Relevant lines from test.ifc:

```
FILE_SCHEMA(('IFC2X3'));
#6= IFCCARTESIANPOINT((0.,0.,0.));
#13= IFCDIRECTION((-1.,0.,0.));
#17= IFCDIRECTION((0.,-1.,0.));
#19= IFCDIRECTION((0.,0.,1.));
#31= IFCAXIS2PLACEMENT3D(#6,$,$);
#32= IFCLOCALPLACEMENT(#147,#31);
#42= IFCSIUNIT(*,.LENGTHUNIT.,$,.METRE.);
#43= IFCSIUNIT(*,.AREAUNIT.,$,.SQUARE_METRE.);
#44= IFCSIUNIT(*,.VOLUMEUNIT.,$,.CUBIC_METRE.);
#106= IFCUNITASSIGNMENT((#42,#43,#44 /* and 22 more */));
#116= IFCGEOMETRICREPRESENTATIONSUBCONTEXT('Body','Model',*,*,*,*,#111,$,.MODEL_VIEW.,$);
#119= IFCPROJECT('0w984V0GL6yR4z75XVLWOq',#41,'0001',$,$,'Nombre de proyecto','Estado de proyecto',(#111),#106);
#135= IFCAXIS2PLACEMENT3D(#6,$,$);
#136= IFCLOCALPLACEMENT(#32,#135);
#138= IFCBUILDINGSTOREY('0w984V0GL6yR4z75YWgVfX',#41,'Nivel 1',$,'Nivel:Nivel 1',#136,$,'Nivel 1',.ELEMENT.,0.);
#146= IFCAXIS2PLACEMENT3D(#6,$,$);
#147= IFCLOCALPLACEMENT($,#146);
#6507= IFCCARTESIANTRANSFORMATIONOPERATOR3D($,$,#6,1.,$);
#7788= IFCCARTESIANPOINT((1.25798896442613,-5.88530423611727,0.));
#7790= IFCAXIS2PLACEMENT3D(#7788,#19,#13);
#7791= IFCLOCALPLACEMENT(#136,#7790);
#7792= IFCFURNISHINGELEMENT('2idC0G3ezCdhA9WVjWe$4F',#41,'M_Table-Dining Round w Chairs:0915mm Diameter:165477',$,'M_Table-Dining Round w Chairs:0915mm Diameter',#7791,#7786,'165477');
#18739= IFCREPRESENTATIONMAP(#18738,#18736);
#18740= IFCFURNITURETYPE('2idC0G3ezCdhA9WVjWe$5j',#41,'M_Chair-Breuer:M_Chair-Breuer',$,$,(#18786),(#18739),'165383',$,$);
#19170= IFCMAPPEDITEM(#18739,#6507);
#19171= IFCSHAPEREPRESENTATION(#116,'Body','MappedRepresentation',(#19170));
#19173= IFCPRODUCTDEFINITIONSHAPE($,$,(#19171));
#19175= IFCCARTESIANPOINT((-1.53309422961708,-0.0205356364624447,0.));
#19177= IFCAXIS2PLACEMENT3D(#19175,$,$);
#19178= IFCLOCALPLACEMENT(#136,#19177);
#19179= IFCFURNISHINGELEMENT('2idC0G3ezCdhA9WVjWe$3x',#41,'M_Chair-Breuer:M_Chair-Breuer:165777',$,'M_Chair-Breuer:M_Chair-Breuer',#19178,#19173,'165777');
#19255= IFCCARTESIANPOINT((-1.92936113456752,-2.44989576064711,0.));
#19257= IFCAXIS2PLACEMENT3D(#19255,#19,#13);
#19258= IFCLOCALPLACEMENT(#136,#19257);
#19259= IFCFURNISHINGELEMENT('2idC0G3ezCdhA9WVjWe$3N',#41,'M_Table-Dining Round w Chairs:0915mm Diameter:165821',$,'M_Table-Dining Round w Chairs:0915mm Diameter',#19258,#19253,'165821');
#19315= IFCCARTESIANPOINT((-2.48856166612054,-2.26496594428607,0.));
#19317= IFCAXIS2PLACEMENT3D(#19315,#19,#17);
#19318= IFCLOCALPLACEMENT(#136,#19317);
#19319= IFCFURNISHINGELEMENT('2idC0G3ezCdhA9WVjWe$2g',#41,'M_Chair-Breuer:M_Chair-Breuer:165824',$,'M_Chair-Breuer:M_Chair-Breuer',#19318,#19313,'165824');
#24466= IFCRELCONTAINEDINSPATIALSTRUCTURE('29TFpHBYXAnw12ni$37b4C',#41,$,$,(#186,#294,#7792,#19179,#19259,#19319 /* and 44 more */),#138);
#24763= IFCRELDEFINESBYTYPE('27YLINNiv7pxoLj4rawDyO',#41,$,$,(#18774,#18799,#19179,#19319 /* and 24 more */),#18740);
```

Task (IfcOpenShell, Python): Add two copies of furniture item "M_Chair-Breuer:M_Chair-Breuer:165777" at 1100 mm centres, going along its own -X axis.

```python
import ifcopenshell
import ifcopenshell.api.geometry
import ifcopenshell.api.root
import ifcopenshell.util.element
import ifcopenshell.util.placement
import ifcopenshell.util.unit

model = ifcopenshell.open("test.ifc")
unit_scale = ifcopenshell.util.unit.calculate_unit_scale(model)


def reuse_history(source, copy):
    """copy_class also copies each property set's owner history, people and application; keep the originals."""
    for rel in copy.IsDefinedBy:
        if rel.is_a("IfcRelDefinesByProperties") and (history := rel.RelatingPropertyDefinition.OwnerHistory):
            rel.RelatingPropertyDefinition.OwnerHistory = source.OwnerHistory
            ifcopenshell.util.element.remove_deep2(model, history)


source = model.by_id(19179)
base = ifcopenshell.util.placement.get_local_placement(source.ObjectPlacement)
step = -base[:3, 0] * 1.1 / unit_scale

for i in range(1, 3):
    copy = ifcopenshell.api.root.copy_class(model, product=source)
    copy.Representation = ifcopenshell.util.element.copy_deep(
        model, source.Representation, exclude=["IfcGeometricRepresentationContext", "IfcRepresentationMap"]
    )
    copy.Name = "M_Chair-Breuer:M_Chair-Breuer"
    copy.Tag = None
    reuse_history(source, copy)
    matrix = base.copy()
    matrix[:3, 3] += i * step
    print("added at", matrix[:3, 3].round(3) + 0.0)
    ifcopenshell.api.geometry.edit_object_placement(model, product=copy, matrix=matrix, is_si=False)

model.write("test_updated.ifc")
```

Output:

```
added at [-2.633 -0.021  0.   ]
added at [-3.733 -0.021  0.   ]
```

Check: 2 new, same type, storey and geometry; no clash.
